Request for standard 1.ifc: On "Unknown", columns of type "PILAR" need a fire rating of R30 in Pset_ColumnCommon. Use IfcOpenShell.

First a look at what the model holds.

```python
import ifcopenshell
import ifcopenshell.util.element

model = ifcopenshell.open("standard 1.ifc")
print(model.schema)
storey = next(s for s in model.by_type("IfcBuildingStorey") if s.Name == "Unknown")
columns = [e for e in ifcopenshell.util.element.get_decomposition(storey) if e.is_a("IfcColumn")]
seen = {}
for e in columns:
    element_type = ifcopenshell.util.element.get_type(e)
    key = (element_type.Name if element_type != e and element_type else None, ifcopenshell.util.element.get_pset(e, "Pset_ColumnCommon", "FireRating"))
    seen[key] = seen.get(key, 0) + 1
for (name, value), count in sorted(seen.items(), key=str):
    print(count, "x", name, "|", value)
```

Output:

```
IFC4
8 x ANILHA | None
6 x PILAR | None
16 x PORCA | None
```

```python
import ifcopenshell
import ifcopenshell.api.pset
import ifcopenshell.util.element

model = ifcopenshell.open("standard 1.ifc")

storey = next(s for s in model.by_type("IfcBuildingStorey") if s.Name == "Unknown")
columns = [e for e in ifcopenshell.util.element.get_decomposition(storey) if e.is_a("IfcColumn")]

count = 0
for e in columns:
    element_type = ifcopenshell.util.element.get_type(e)
    if element_type in (None, e) or element_type.Name != "PILAR":
        continue
    found = ifcopenshell.util.element.get_pset(e, "Pset_ColumnCommon", should_inherit=False)
    if found:
        pset = model.by_id(found["id"])
        if len(ifcopenshell.util.element.get_elements_by_pset(pset)) > 1:
            pset = ifcopenshell.api.pset.unshare_pset(model, products=[e], pset=pset)[0]
    else:
        pset = ifcopenshell.api.pset.add_pset(model, product=e, name="Pset_ColumnCommon")
    ifcopenshell.api.pset.edit_pset(model, pset=pset, properties={"FireRating": "R30"})
    count += 1

print(count, "columns updated")

model.write("standard 1_rev.ifc")
```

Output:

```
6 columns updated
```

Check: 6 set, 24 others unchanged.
